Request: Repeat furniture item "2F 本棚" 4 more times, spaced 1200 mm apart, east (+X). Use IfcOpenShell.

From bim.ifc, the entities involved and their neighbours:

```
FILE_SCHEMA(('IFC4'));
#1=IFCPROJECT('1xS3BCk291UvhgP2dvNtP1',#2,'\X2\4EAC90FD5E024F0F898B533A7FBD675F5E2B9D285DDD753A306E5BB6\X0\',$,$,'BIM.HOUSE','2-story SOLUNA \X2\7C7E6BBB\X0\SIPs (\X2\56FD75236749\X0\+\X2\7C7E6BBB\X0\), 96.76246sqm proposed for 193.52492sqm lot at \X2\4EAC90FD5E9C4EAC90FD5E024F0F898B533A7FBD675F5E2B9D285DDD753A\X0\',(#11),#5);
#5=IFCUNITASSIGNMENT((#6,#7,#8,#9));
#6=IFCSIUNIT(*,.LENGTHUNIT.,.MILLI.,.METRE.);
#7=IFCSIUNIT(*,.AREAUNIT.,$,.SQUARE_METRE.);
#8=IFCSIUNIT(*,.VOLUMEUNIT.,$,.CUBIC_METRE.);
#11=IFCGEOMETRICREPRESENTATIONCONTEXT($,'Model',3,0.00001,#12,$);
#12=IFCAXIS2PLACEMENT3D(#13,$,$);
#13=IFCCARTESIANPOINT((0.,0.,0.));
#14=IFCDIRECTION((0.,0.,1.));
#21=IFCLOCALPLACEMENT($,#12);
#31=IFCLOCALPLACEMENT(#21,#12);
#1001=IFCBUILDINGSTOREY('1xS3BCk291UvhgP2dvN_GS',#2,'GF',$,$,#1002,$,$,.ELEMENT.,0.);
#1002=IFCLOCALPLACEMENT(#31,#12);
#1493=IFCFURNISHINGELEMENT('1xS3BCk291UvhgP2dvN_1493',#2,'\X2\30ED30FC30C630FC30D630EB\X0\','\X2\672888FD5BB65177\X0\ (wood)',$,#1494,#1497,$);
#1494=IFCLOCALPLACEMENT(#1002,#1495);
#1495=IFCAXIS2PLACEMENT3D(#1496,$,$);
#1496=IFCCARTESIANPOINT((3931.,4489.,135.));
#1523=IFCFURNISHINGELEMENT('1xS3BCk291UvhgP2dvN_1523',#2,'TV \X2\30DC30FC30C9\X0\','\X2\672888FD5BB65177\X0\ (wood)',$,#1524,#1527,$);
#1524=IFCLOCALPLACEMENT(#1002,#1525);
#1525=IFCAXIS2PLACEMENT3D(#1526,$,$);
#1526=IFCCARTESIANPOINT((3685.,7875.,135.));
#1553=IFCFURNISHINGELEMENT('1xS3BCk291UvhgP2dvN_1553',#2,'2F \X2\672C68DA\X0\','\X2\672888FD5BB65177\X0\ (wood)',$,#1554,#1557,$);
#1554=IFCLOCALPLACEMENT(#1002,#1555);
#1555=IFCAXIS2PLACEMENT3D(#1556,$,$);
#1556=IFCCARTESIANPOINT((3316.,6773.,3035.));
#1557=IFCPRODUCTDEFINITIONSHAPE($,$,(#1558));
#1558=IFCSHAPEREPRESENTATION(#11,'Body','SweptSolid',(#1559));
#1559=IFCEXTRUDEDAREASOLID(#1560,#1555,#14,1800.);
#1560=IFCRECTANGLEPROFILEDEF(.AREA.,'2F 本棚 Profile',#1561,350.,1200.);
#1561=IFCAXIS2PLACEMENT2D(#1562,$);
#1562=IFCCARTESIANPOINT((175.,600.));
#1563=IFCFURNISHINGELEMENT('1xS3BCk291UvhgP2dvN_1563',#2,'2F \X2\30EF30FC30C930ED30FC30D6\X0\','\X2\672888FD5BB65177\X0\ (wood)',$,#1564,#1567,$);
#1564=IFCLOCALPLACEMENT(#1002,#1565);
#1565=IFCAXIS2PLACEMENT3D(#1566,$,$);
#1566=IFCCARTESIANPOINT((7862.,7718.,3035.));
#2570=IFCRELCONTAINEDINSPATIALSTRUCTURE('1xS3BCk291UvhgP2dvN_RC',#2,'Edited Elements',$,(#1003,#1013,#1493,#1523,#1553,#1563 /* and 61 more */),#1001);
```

```python
import numpy as np
import ifcopenshell
import ifcopenshell.api.geometry
import ifcopenshell.api.root
import ifcopenshell.util.element
import ifcopenshell.util.placement

model = ifcopenshell.open("bim.ifc")


def reuse_history(source, copy):
    """copy_class also copies each property set's owner history, people and application; keep the originals."""
    for rel in copy.IsDefinedBy:
        if rel.is_a("IfcRelDefinesByProperties") and (history := rel.RelatingPropertyDefinition.OwnerHistory):
            rel.RelatingPropertyDefinition.OwnerHistory = source.OwnerHistory
            ifcopenshell.util.element.remove_deep2(model, history)


source = model.by_guid("1xS3BCk291UvhgP2dvN_1553")
base = ifcopenshell.util.placement.get_local_placement(source.ObjectPlacement)
step = np.array([1.0, 0.0, 0.0]) * 1200.0

for i in range(1, 5):
    copy = ifcopenshell.api.root.copy_class(model, product=source)
    copy.Representation = ifcopenshell.util.element.copy_deep(
        model, source.Representation, exclude=["IfcGeometricRepresentationContext", "IfcRepresentationMap"]
    )
    reuse_history(source, copy)
    matrix = base.copy()
    matrix[:3, 3] += i * step
    print("added at", matrix[:3, 3].round(3) + 0.0)
    ifcopenshell.api.geometry.edit_object_placement(model, product=copy, matrix=matrix, is_si=False)

model.write("bim_updated.ifc")
```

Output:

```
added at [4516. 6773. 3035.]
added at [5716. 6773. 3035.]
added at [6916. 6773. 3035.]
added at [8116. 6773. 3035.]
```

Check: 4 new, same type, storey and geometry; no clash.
